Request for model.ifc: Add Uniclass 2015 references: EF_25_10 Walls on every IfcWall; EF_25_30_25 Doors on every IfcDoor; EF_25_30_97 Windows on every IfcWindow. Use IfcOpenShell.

First a look at what the model holds.

```python
import ifcopenshell

model = ifcopenshell.open("model.ifc")
print(model.schema)
print("classifications:", [c.Name for c in model.by_type("IfcClassification")])
for ifc_class in ("IfcDoor", "IfcRoof", "IfcStair", "IfcWall", "IfcWindow"):
    print(ifc_class, len(model.by_type(ifc_class)))
```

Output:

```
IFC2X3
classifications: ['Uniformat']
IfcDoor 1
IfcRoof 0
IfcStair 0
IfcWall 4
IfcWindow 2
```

```python
import ifcopenshell
import ifcopenshell.api.classification

model = ifcopenshell.open("model.ifc")

# IFC2X3 requires Source and Edition and has no link from the project to the system.
system = model.create_entity("IfcClassification", Source="NBS", Edition="2015", Name="Uniclass 2015")

codes = {
    "IfcWall": ("EF_25_10", "Walls"),
    "IfcDoor": ("EF_25_30_25", "Doors"),
    "IfcWindow": ("EF_25_30_97", "Windows"),
}
for ifc_class, (code, name) in codes.items():
    products = model.by_type(ifc_class)
    ifcopenshell.api.classification.add_reference(
        model, products=products, classification=system, identification=code, name=name
    )
    print(code, len(products))

model.write("model-out.ifc")
```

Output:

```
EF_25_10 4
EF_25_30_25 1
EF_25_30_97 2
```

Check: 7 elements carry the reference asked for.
